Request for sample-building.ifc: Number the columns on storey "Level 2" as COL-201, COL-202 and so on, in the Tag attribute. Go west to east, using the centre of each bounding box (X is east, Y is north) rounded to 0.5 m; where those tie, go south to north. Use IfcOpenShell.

First a look at what the model holds.

```python
import ifcopenshell
import ifcopenshell.util.element
import ifcopenshell.util.placement

model = ifcopenshell.open("sample-building.ifc")
print(model.schema)
storey = next(s for s in model.by_type("IfcBuildingStorey") if s.Name == "Level 2")
columns = [e for e in ifcopenshell.util.element.get_decomposition(storey) if e.is_a("IfcColumn")]
for e in sorted(columns, key=lambda e: e.id()):
    origin = ifcopenshell.util.placement.get_local_placement(e.ObjectPlacement)[:3, 3]
    print(e.id(), e.Tag, e.Name, origin.round(2) + 0.0, sep=" | ")
```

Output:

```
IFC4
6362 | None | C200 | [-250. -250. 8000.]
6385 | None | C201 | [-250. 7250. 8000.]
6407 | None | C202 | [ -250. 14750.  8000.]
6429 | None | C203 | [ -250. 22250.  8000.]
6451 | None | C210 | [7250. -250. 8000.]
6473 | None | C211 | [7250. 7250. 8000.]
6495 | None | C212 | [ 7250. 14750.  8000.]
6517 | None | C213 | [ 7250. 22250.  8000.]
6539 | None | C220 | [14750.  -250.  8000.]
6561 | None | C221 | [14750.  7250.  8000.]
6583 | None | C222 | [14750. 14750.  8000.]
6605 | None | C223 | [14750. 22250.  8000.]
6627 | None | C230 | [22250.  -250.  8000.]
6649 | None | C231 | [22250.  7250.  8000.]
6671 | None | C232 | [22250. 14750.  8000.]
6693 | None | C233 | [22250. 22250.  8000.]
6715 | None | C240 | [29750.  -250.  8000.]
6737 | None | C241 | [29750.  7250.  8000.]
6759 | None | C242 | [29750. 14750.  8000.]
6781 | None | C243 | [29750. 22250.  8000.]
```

```python
import ifcopenshell
import ifcopenshell.geom
import ifcopenshell.util.element
import ifcopenshell.util.shape

model = ifcopenshell.open("sample-building.ifc")
settings = ifcopenshell.geom.settings()
settings.set("use-world-coords", True)


def centre(element):
    shape = ifcopenshell.geom.create_shape(settings, element)
    return ifcopenshell.util.shape.get_bbox_centroid(shape.geometry)


storey = next(s for s in model.by_type("IfcBuildingStorey") if s.Name == "Level 2")
columns = [e for e in ifcopenshell.util.element.get_decomposition(storey) if e.is_a("IfcColumn")]

# Insertion points can sit at a corner or the storey origin, so sort by the geometry (in metres).
centres = {e: centre(e) for e in columns}
columns.sort(key=lambda e: (round(centres[e][0] / 0.5), centres[e][1]))

for i, e in enumerate(columns, start=1):
    number = f"COL-2{i:02d}"
    e.Tag = number
    print(e.id(), number)

model.write("sample-building_v2.ifc")
```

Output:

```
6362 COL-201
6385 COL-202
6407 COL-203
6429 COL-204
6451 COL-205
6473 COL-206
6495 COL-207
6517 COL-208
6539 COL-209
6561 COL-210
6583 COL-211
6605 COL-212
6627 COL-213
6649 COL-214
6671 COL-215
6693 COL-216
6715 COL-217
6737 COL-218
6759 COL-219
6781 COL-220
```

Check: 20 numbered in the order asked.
